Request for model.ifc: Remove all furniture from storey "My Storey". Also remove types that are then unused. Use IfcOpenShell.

First a look at what the model holds.

```python
import ifcopenshell
import ifcopenshell.util.element

model = ifcopenshell.open("model.ifc")
print(model.schema)
storey = next(s for s in model.by_type("IfcBuildingStorey") if s.Name == "My Storey")
furniture = [e for e in ifcopenshell.util.element.get_decomposition(storey) if e.is_a("IfcFurnishingElement")]
seen = {}
for e in furniture:
    element_type = ifcopenshell.util.element.get_type(e)
    name = element_type.Name if element_type not in (None, e) else None
    seen[name] = seen.get(name, 0) + 1
for name, count in sorted(seen.items(), key=str):
    print(count, "x", name)
```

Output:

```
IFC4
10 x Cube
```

```python
import ifcopenshell
import ifcopenshell.api.root
import ifcopenshell.util.element

model = ifcopenshell.open("model.ifc")

storey = next(s for s in model.by_type("IfcBuildingStorey") if s.Name == "My Storey")
furniture = [e for e in ifcopenshell.util.element.get_decomposition(storey) if e.is_a("IfcFurnishingElement")]
types = {ifcopenshell.util.element.get_type(e) for e in furniture} - {None, *furniture}

for e in furniture:
    ifcopenshell.api.root.remove_product(model, product=e)
print(len(furniture), "removed")

unused = [t for t in types if not ifcopenshell.util.element.get_types(t)]
for t in unused:
    ifcopenshell.api.root.remove_product(model, product=t)
print(len(unused), "unused types removed")

model.write("model_edited.ifc")
```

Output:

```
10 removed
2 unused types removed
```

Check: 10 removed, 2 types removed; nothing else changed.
